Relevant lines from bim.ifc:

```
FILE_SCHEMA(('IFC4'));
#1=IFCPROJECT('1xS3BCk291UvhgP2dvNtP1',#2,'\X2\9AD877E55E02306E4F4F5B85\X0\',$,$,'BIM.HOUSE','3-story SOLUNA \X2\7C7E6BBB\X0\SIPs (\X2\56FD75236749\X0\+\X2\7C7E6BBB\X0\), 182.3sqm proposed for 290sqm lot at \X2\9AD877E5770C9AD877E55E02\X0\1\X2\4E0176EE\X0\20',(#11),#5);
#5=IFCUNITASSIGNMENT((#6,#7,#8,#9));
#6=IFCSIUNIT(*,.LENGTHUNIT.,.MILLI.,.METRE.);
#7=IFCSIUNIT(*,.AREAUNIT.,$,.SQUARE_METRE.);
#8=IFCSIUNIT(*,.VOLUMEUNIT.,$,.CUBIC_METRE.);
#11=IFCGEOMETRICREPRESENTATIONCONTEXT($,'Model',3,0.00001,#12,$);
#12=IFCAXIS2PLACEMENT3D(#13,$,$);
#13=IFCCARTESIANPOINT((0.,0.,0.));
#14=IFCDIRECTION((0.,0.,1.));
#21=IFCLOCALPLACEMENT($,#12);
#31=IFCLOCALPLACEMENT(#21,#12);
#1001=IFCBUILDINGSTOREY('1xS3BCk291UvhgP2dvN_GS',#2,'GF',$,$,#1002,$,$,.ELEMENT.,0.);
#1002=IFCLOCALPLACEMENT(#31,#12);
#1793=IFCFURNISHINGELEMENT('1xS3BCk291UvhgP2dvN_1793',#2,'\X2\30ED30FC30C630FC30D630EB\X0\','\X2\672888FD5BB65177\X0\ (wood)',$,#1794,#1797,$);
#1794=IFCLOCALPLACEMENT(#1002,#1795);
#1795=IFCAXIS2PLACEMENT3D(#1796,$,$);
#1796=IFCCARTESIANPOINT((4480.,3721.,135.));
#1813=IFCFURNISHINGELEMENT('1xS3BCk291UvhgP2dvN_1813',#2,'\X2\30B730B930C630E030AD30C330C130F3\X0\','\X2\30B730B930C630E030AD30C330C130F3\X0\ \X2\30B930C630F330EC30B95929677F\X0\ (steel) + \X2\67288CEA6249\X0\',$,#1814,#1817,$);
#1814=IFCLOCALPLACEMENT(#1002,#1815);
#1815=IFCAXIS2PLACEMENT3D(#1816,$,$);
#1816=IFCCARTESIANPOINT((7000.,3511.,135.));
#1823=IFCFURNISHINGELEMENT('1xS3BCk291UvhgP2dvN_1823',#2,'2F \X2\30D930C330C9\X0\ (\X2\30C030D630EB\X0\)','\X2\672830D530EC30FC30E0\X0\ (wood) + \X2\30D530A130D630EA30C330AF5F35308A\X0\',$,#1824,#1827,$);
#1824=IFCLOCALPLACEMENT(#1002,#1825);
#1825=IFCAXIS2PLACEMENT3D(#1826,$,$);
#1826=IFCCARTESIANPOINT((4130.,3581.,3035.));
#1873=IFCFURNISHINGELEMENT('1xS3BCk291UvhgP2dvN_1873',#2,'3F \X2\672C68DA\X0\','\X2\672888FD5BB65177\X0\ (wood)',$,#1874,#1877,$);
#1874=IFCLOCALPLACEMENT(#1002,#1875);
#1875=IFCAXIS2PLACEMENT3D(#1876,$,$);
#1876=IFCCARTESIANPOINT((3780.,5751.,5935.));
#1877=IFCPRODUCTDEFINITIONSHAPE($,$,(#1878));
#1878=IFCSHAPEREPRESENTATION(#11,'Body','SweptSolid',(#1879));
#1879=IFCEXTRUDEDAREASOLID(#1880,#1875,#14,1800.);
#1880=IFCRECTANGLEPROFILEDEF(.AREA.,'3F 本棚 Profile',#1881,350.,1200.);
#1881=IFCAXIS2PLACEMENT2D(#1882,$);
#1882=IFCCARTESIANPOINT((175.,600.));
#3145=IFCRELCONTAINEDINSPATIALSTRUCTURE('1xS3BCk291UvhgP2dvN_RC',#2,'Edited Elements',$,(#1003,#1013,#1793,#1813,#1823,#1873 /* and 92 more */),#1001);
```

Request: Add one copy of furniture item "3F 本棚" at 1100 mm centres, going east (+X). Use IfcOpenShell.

```python
import numpy as np
import ifcopenshell
import ifcopenshell.api.geometry
import ifcopenshell.api.root
import ifcopenshell.util.element
import ifcopenshell.util.placement
import ifcopenshell.util.unit

model = ifcopenshell.open("bim.ifc")
unit_scale = ifcopenshell.util.unit.calculate_unit_scale(model)


def reuse_history(source, copy):
    """copy_class also copies each property set's owner history, people and application; keep the originals."""
    for rel in copy.IsDefinedBy:
        if rel.is_a("IfcRelDefinesByProperties") and (history := rel.RelatingPropertyDefinition.OwnerHistory):
            rel.RelatingPropertyDefinition.OwnerHistory = source.OwnerHistory
            ifcopenshell.util.element.remove_deep2(model, history)


source = model.by_guid("1xS3BCk291UvhgP2dvN_1873")
base = ifcopenshell.util.placement.get_local_placement(source.ObjectPlacement)
step = np.array([1.0, 0.0, 0.0]) * 1.1 / unit_scale

for i in range(1, 2):
    copy = ifcopenshell.api.root.copy_class(model, product=source)
    copy.Representation = ifcopenshell.util.element.copy_deep(
        model, source.Representation, exclude=["IfcGeometricRepresentationContext", "IfcRepresentationMap"]
    )
    reuse_history(source, copy)
    matrix = base.copy()
    matrix[:3, 3] += i * step
    print("added at", matrix[:3, 3].round(3) + 0.0)
    ifcopenshell.api.geometry.edit_object_placement(model, product=copy, matrix=matrix, is_si=False)

model.write("bim-out.ifc")
```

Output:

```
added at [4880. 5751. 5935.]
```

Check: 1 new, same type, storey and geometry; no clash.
